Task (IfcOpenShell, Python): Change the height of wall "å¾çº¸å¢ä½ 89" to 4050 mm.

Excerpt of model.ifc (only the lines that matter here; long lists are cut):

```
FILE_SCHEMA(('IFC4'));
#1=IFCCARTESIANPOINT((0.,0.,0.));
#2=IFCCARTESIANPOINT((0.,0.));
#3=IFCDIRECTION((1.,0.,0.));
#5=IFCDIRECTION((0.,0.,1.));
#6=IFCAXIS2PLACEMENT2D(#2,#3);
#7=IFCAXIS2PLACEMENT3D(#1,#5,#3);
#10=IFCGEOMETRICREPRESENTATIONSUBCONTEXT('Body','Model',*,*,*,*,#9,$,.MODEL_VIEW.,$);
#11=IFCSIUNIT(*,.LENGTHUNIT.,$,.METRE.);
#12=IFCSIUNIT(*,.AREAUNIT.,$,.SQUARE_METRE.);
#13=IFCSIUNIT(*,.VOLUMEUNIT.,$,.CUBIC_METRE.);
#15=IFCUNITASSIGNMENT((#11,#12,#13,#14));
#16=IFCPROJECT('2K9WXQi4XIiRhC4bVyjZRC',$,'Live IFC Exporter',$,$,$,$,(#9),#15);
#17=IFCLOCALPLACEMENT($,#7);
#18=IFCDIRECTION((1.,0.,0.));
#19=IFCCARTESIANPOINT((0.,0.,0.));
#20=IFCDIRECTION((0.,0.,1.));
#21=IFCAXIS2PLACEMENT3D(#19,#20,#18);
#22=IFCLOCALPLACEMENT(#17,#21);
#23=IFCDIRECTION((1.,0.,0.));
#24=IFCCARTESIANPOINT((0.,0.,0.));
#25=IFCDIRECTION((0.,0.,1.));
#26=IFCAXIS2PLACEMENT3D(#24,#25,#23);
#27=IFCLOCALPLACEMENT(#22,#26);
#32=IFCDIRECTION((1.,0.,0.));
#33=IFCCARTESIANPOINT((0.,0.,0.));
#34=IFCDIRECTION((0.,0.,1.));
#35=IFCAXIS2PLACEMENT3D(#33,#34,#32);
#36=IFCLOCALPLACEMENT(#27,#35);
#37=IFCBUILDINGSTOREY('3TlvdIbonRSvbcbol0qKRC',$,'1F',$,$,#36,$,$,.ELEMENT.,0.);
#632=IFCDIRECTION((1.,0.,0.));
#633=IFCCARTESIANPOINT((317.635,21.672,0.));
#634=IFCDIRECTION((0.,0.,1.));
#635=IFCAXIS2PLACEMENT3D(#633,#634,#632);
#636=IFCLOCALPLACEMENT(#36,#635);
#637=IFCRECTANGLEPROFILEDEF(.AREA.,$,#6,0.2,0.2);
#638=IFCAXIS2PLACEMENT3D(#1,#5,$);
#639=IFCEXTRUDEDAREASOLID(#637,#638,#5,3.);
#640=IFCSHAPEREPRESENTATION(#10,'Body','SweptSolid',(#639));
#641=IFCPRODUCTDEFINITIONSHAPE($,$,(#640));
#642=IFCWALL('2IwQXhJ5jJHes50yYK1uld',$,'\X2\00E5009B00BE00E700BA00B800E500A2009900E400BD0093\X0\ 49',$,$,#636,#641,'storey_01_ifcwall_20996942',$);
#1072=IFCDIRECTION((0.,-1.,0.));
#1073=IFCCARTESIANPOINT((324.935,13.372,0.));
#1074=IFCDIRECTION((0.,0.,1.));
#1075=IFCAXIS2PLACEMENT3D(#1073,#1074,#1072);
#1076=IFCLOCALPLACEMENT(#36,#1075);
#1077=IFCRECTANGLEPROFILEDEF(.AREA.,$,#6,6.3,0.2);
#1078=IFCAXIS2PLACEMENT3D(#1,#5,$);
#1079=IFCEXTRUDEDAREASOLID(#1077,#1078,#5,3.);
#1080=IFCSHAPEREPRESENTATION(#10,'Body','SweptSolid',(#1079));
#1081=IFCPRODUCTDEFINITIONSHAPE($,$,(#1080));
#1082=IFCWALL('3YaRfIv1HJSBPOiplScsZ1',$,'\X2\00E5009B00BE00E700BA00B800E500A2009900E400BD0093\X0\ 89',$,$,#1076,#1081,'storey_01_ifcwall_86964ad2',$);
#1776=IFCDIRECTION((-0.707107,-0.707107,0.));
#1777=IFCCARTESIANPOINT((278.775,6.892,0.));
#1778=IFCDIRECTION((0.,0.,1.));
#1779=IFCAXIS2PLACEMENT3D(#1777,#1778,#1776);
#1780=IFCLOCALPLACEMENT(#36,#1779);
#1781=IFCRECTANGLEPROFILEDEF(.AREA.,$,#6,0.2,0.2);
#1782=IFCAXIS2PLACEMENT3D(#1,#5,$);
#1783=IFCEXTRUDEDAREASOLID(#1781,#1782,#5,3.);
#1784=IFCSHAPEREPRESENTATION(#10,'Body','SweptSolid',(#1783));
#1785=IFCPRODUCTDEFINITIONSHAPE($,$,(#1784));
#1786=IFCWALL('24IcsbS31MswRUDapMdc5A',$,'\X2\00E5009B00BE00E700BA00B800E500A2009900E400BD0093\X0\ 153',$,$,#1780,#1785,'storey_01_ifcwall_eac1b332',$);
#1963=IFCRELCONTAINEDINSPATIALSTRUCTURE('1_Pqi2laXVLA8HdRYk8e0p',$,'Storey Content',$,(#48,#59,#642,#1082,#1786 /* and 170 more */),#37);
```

```python
import ifcopenshell
import ifcopenshell.geom
import ifcopenshell.util.representation
import ifcopenshell.util.shape

model = ifcopenshell.open("model.ifc")
settings = ifcopenshell.geom.settings()


def volume(element):
    """Net volume in cubic metres, openings subtracted."""
    shape = ifcopenshell.geom.create_shape(settings, element)
    return ifcopenshell.util.shape.get_volume(shape.geometry)


wall = model.by_guid("3YaRfIv1HJSBPOiplScsZ1")
before = volume(wall)

body = ifcopenshell.util.representation.get_representation(wall, "Model", "Body")
solid = body.Items[0]
old_height = solid.Depth
solid.Depth = 4.05
after = volume(wall)

print(f"height {old_height:g} -> {solid.Depth:g}, volume {before:.3f} -> {after:.3f} m3")

model.write("model_edited.ifc")
```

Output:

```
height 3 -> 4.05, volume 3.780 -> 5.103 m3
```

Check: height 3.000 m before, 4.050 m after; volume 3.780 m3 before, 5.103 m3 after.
